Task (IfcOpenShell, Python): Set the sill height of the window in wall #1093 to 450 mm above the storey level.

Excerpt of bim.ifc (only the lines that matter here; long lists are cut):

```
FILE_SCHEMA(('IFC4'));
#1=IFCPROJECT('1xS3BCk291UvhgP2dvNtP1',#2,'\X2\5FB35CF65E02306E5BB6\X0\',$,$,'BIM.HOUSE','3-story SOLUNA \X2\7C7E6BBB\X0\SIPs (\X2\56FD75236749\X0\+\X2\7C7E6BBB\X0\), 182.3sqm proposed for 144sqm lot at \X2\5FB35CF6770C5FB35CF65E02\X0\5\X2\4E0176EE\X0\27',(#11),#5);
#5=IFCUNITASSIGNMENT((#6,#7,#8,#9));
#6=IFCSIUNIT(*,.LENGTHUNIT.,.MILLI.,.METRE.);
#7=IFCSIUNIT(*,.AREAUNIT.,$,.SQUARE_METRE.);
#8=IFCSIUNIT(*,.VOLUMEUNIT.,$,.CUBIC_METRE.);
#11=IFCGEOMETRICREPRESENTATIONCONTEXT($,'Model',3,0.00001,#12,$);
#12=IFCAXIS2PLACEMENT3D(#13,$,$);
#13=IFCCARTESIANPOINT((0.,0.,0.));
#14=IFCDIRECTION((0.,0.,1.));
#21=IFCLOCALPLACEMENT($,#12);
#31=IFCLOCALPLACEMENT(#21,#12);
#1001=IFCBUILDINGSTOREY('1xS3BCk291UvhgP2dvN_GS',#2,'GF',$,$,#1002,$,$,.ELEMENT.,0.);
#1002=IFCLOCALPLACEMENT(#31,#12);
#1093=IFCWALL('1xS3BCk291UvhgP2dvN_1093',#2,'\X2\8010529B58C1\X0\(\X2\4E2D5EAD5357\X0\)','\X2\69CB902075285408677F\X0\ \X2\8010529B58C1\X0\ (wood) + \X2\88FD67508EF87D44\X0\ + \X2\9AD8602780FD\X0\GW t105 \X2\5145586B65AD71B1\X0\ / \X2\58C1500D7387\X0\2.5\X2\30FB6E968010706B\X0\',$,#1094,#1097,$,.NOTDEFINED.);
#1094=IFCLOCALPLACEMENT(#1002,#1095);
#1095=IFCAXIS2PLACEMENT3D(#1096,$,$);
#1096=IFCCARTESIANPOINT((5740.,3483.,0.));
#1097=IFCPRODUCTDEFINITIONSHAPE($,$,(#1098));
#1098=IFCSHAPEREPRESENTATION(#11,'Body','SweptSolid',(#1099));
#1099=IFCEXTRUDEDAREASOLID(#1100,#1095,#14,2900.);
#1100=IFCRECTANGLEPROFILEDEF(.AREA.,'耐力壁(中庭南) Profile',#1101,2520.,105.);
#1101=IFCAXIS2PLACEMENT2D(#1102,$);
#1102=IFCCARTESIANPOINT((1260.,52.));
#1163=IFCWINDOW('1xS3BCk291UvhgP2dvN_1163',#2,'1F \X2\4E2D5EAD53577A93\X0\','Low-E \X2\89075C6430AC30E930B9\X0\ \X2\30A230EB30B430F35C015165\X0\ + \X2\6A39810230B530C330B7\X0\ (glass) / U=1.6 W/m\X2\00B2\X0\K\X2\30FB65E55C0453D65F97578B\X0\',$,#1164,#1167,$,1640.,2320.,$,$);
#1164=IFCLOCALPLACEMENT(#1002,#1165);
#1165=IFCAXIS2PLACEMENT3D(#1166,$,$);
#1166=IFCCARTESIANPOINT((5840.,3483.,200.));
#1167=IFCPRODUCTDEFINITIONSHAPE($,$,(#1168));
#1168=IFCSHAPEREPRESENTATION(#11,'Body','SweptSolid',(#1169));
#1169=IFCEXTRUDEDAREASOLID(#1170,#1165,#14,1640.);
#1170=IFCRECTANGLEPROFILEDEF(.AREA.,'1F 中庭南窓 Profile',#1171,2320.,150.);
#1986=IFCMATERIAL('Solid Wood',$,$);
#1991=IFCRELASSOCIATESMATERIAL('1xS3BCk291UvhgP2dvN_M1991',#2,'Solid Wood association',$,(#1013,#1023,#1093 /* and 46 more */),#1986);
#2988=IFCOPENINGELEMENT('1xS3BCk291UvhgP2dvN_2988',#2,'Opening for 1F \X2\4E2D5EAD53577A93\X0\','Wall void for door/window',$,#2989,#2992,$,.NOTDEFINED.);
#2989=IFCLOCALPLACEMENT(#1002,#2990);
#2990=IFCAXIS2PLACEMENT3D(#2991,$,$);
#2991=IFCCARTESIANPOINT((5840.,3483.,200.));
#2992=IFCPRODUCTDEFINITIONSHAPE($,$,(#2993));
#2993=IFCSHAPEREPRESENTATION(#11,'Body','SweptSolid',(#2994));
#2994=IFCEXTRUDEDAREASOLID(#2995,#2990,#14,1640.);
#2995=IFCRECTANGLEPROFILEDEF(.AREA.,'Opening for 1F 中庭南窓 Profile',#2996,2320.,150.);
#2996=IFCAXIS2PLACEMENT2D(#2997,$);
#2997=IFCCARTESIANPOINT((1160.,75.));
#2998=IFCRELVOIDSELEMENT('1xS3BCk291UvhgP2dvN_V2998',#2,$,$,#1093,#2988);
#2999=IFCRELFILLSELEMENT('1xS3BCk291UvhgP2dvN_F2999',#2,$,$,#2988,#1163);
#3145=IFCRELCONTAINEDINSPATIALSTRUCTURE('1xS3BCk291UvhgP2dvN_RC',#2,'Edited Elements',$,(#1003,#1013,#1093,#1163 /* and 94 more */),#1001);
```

```python
import numpy as np
import ifcopenshell
import ifcopenshell.api.geometry
import ifcopenshell.geom
import ifcopenshell.util.element
import ifcopenshell.util.placement
import ifcopenshell.util.shape
import ifcopenshell.util.unit

model = ifcopenshell.open("bim.ifc")
unit_scale = ifcopenshell.util.unit.calculate_unit_scale(model)

window = model.by_guid("1xS3BCk291UvhgP2dvN_1163")
opening = window.FillsVoids[0].RelatingOpeningElement
storey = ifcopenshell.util.element.get_container(window, ifc_class="IfcBuildingStorey")
level = ifcopenshell.util.placement.get_local_placement(storey.ObjectPlacement)[2, 3]

# The opening's origin need not be at the sill, so measure its lowest point.
shape = ifcopenshell.geom.create_shape(ifcopenshell.geom.settings(), opening)
bottom = ifcopenshell.util.shape.get_shape_bottom_elevation(shape, shape.geometry) / unit_scale
dz = level + 450.0 - bottom

shift = np.array([0.0, 0.0, dz])
# The window is not placed relative to its opening, so move both.
for product in (opening, window):
    matrix = ifcopenshell.util.placement.get_local_placement(product.ObjectPlacement)
    matrix[:3, 3] += shift
    ifcopenshell.api.geometry.edit_object_placement(model, product=product, matrix=matrix, is_si=False)

print(f"moved by {dz * unit_scale:+.3f} m")

model.write("bim_rev.ifc")
```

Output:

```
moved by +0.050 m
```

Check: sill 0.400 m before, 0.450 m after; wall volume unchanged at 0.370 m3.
